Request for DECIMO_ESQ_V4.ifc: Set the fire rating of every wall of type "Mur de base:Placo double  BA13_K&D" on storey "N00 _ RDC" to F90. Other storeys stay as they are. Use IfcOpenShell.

First a look at what the model holds.

```python
import ifcopenshell
import ifcopenshell.util.element

model = ifcopenshell.open("DECIMO_ESQ_V4.ifc")
print(model.schema)
storey = next(s for s in model.by_type("IfcBuildingStorey") if s.Name == "N00 _ RDC")
walls = [e for e in ifcopenshell.util.element.get_decomposition(storey) if e.is_a("IfcWall")]
seen = {}
for e in walls:
    element_type = ifcopenshell.util.element.get_type(e)
    key = (element_type.Name if element_type != e and element_type else None, ifcopenshell.util.element.get_pset(e, "Pset_WallCommon", "FireRating"))
    seen[key] = seen.get(key, 0) + 1
for (name, value), count in sorted(seen.items(), key=str):
    print(count, "x", name, "|", value)
```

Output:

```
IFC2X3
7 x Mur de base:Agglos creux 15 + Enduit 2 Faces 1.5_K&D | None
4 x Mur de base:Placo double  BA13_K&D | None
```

```python
import ifcopenshell
import ifcopenshell.api.pset
import ifcopenshell.util.element

model = ifcopenshell.open("DECIMO_ESQ_V4.ifc")

storey = next(s for s in model.by_type("IfcBuildingStorey") if s.Name == "N00 _ RDC")
walls = [e for e in ifcopenshell.util.element.get_decomposition(storey) if e.is_a("IfcWall")]

count = 0
for e in walls:
    element_type = ifcopenshell.util.element.get_type(e)
    if element_type in (None, e) or element_type.Name != "Mur de base:Placo double  BA13_K&D":
        continue
    # add_pset returns the element's existing set when there is one.
    pset = ifcopenshell.api.pset.add_pset(model, product=e, name="Pset_WallCommon")
    ifcopenshell.api.pset.edit_pset(model, pset=pset, properties={"FireRating": "F90"})
    count += 1

print(count, "walls updated")

model.write("DECIMO_ESQ_V4_edited.ifc")
```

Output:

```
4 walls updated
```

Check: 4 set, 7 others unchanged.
